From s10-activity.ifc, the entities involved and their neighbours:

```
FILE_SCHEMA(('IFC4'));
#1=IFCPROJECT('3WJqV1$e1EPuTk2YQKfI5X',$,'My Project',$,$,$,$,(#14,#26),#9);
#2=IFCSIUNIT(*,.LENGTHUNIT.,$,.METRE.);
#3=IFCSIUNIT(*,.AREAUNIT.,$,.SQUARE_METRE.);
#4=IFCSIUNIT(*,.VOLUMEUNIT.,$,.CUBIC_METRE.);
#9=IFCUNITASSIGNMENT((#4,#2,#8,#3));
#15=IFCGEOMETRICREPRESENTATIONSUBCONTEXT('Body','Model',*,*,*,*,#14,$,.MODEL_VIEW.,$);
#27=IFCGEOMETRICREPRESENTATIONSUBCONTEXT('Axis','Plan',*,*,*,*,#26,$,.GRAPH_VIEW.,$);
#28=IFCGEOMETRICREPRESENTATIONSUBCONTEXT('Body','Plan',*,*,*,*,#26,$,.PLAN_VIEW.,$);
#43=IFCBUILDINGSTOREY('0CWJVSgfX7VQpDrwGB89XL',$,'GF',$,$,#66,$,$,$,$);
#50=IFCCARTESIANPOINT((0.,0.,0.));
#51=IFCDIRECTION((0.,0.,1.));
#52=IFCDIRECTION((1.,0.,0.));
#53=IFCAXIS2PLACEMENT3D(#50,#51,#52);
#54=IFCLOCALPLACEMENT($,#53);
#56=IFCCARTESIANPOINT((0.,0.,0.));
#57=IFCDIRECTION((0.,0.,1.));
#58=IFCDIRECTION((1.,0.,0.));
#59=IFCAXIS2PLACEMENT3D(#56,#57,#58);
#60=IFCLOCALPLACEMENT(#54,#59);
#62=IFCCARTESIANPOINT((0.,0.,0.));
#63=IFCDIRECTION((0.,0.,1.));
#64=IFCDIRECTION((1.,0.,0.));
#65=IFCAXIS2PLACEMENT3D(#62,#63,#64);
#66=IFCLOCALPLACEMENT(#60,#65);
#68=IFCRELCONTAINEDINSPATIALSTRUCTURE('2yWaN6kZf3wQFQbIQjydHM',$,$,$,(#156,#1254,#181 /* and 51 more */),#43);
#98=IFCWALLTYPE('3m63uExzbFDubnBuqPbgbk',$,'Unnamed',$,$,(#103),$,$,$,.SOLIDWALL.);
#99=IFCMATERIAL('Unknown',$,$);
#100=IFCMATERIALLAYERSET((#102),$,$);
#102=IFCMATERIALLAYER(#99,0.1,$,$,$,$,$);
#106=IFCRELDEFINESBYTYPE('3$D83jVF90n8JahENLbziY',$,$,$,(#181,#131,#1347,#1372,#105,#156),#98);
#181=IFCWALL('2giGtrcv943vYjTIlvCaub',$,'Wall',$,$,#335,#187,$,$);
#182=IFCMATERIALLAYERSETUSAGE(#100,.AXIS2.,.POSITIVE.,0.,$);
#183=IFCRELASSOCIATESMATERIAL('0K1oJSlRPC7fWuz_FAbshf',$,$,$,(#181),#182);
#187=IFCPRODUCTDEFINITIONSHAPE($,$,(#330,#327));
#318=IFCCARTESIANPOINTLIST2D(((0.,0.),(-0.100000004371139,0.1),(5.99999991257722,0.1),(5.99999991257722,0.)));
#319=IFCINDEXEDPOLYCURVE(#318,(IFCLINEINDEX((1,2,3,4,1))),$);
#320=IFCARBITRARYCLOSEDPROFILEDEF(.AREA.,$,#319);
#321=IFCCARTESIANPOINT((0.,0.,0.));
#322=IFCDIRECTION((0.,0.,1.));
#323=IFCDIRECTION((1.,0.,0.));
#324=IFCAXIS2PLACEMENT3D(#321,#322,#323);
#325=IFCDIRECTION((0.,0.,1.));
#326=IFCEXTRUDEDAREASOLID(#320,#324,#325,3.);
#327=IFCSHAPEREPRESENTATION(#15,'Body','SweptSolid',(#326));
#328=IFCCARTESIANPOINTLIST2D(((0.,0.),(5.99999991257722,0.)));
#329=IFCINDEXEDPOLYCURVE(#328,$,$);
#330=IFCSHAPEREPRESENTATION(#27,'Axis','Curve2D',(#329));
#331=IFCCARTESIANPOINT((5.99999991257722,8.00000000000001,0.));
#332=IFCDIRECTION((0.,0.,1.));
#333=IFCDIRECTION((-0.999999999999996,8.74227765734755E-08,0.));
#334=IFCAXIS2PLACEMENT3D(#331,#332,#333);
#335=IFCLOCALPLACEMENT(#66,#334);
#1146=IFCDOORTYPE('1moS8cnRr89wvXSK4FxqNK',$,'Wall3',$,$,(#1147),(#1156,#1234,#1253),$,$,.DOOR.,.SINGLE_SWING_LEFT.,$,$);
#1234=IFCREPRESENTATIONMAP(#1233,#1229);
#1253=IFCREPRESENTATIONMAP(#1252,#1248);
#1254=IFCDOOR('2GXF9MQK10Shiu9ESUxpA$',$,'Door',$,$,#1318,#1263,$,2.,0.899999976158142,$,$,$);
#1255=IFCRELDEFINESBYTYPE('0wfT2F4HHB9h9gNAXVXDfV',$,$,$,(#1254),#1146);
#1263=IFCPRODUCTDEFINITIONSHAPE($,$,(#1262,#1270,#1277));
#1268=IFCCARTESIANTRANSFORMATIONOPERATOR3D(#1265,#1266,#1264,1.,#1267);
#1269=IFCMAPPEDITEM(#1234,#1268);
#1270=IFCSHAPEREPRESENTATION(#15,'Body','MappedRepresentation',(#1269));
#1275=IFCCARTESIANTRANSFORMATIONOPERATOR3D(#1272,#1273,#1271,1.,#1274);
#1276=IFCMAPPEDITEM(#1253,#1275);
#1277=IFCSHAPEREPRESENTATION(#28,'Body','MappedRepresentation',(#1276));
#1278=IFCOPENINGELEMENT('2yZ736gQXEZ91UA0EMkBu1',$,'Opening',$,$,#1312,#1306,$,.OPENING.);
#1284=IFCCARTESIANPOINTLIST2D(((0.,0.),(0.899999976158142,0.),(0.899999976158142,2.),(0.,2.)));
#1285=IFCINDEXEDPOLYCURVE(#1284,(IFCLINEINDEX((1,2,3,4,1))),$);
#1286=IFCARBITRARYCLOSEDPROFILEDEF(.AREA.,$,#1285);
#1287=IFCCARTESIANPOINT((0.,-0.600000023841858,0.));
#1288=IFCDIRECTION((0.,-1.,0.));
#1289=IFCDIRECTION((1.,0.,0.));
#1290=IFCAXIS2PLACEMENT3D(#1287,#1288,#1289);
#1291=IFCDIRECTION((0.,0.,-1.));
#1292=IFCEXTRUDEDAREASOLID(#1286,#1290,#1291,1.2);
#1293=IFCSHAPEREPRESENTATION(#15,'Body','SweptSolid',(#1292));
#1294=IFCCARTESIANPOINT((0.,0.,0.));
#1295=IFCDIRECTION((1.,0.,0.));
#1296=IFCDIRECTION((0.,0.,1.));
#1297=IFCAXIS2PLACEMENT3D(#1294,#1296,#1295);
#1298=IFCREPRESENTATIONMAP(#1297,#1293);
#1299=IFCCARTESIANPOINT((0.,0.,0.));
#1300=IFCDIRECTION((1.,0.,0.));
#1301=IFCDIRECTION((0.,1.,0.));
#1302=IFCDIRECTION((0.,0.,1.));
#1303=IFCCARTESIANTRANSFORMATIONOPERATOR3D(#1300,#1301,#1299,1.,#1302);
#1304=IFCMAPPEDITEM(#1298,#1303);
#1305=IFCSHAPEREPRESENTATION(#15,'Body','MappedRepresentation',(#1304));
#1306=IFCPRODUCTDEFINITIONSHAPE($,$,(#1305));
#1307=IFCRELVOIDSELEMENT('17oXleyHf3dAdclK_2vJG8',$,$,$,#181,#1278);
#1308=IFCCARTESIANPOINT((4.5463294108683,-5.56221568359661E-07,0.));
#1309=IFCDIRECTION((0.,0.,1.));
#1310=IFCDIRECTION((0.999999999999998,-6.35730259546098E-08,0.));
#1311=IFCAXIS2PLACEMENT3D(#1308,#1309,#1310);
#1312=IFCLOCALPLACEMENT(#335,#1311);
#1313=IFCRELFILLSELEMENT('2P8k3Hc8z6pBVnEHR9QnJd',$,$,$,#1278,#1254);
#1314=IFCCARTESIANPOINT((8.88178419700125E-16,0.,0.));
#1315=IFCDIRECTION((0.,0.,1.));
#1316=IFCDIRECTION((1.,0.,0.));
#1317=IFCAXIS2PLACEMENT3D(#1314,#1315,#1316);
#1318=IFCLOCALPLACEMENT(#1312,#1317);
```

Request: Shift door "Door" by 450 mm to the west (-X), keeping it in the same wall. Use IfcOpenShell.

```python
import ifcopenshell
import ifcopenshell.api.geometry
import ifcopenshell.util.placement

model = ifcopenshell.open("s10-activity.ifc")

door = model.by_id(1254)
opening = door.FillsVoids[0].RelatingOpeningElement
wall = opening.VoidsElements[0].RelatingBuildingElement

wall_matrix = ifcopenshell.util.placement.get_local_placement(wall.ObjectPlacement)
shift = wall_matrix[:3, 0] * 0.45
before = ifcopenshell.util.placement.get_local_placement(door.ObjectPlacement)[:3, 3].copy()

# The door is placed relative to its opening, so it follows when the opening moves.
matrix = ifcopenshell.util.placement.get_local_placement(opening.ObjectPlacement)
matrix[:3, 3] += shift
ifcopenshell.api.geometry.edit_object_placement(
    model, product=opening, matrix=matrix, is_si=False, should_transform_children=True
)

after = ifcopenshell.util.placement.get_local_placement(door.ObjectPlacement)[:3, 3]
print("door moved by", (after - before).round(3) + 0.0)

model.write("s10-activity-out.ifc")
```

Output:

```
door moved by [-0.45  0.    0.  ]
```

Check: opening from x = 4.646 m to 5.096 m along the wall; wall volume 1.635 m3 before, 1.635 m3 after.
